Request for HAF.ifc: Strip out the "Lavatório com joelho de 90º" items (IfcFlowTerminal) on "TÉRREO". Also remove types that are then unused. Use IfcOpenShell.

First a look at what the model holds.

```python
import ifcopenshell
import ifcopenshell.util.element

model = ifcopenshell.open("HAF.ifc")
print(model.schema)
storey = next(s for s in model.by_type("IfcBuildingStorey") if s.Name == "TÉRREO")
terminals = [e for e in ifcopenshell.util.element.get_decomposition(storey) if e.is_a("IfcFlowTerminal")]
seen = {}
for e in terminals:
    element_type = ifcopenshell.util.element.get_type(e)
    name = element_type.Name if element_type not in (None, e) else None
    seen[name] = seen.get(name, 0) + 1
for name, count in sorted(seen.items(), key=str):
    print(count, "x", name)
```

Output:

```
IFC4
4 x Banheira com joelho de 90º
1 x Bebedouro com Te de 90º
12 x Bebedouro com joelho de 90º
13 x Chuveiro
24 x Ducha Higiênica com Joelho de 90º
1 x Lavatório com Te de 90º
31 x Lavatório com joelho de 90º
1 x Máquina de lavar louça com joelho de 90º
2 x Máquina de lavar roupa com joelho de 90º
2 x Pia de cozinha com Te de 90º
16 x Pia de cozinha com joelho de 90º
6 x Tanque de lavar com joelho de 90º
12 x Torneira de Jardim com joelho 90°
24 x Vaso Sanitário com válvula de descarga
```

```python
import ifcopenshell
import ifcopenshell.api.root
import ifcopenshell.util.element

model = ifcopenshell.open("HAF.ifc")

storey = next(s for s in model.by_type("IfcBuildingStorey") if s.Name == "TÉRREO")
terminals = [e for e in ifcopenshell.util.element.get_decomposition(storey) if e.is_a("IfcFlowTerminal")]
targets = [e for e in terminals if (t := ifcopenshell.util.element.get_type(e)) not in (None, e) and t.Name == "Lavatório com joelho de 90º"]
types = {ifcopenshell.util.element.get_type(e) for e in targets} - {None, *targets}

for e in targets:
    ifcopenshell.api.root.remove_product(model, product=e)
print(len(targets), "removed")

unused = [t for t in types if not ifcopenshell.util.element.get_types(t)]
for t in unused:
    ifcopenshell.api.root.remove_product(model, product=t)
print(len(unused), "unused types removed")

model.write("HAF-out.ifc")
```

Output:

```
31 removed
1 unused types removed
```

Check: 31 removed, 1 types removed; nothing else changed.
